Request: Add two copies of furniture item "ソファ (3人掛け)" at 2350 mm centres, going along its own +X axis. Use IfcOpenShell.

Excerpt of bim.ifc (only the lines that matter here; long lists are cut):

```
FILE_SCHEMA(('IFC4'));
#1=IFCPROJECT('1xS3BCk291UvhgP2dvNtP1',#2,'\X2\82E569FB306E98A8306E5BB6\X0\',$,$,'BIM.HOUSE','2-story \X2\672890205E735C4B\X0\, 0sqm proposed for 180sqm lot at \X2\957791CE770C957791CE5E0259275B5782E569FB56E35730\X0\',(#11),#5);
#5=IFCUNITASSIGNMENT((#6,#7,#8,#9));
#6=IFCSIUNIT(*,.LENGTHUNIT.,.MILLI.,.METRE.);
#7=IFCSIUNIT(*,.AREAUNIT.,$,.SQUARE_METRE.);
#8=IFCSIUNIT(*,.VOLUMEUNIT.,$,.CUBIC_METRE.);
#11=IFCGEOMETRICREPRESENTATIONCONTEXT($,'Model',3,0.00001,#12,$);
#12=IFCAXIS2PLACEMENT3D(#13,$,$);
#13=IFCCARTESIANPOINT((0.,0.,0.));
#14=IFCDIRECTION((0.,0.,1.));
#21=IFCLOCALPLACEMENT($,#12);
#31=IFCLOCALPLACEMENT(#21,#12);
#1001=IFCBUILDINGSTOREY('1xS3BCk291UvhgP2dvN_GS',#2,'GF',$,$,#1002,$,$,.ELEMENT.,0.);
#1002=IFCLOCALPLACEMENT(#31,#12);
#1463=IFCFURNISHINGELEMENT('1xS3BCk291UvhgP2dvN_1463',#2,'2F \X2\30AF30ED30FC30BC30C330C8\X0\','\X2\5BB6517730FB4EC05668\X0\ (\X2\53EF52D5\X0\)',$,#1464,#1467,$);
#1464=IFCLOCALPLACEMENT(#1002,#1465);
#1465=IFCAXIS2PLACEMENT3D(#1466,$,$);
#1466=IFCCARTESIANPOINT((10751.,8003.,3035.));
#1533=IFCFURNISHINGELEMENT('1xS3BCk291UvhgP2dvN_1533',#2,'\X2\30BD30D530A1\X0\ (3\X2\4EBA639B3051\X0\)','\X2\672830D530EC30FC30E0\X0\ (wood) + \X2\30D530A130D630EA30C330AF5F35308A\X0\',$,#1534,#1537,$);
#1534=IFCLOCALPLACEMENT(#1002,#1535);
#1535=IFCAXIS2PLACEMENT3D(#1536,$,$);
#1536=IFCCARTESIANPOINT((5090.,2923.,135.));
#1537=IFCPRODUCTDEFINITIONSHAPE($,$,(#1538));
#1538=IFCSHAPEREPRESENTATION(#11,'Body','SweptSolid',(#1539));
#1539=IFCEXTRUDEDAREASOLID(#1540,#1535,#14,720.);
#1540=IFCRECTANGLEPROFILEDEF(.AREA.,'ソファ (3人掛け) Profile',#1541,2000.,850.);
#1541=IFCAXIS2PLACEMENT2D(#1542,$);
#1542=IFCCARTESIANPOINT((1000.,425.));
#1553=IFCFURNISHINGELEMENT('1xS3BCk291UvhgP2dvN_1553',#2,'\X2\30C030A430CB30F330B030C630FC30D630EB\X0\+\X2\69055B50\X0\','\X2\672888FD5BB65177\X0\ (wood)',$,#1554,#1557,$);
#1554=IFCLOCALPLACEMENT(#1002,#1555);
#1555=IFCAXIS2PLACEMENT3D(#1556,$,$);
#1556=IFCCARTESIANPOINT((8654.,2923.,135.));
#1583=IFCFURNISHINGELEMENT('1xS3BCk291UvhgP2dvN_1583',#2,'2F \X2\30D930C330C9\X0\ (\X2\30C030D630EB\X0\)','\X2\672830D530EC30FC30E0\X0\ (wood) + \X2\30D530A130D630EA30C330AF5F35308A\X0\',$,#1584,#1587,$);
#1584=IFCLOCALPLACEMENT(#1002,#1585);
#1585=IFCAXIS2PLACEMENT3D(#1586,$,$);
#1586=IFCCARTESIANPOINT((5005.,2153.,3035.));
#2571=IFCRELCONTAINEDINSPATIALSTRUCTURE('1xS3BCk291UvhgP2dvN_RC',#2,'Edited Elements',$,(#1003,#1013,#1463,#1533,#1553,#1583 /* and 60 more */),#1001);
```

```python
import ifcopenshell
import ifcopenshell.api.geometry
import ifcopenshell.api.root
import ifcopenshell.util.element
import ifcopenshell.util.placement
import ifcopenshell.util.unit

model = ifcopenshell.open("bim.ifc")
unit_scale = ifcopenshell.util.unit.calculate_unit_scale(model)


def reuse_history(source, copy):
    """copy_class also copies each property set's owner history, people and application; keep the originals."""
    for rel in copy.IsDefinedBy:
        if rel.is_a("IfcRelDefinesByProperties") and (history := rel.RelatingPropertyDefinition.OwnerHistory):
            rel.RelatingPropertyDefinition.OwnerHistory = source.OwnerHistory
            ifcopenshell.util.element.remove_deep2(model, history)


source = model.by_id(1533)
base = ifcopenshell.util.placement.get_local_placement(source.ObjectPlacement)
step = base[:3, 0] * 2.35 / unit_scale

for i in range(1, 3):
    copy = ifcopenshell.api.root.copy_class(model, product=source)
    copy.Representation = ifcopenshell.util.element.copy_deep(
        model, source.Representation, exclude=["IfcGeometricRepresentationContext", "IfcRepresentationMap"]
    )
    reuse_history(source, copy)
    matrix = base.copy()
    matrix[:3, 3] += i * step
    print("added at", matrix[:3, 3].round(3) + 0.0)
    ifcopenshell.api.geometry.edit_object_placement(model, product=copy, matrix=matrix, is_si=False)

model.write("bim_updated.ifc")
```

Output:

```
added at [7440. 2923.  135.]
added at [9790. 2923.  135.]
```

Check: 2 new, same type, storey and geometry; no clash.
